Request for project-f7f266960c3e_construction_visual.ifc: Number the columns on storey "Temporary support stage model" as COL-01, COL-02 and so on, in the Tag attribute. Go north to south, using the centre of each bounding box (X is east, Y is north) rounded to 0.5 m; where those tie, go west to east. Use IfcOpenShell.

First a look at what the model holds.

```python
import ifcopenshell
import ifcopenshell.util.element
import ifcopenshell.util.placement

model = ifcopenshell.open("project-f7f266960c3e_construction_visual.ifc")
print(model.schema)
storey = next(s for s in model.by_type("IfcBuildingStorey") if s.Name == "Temporary support stage model")
columns = [e for e in ifcopenshell.util.element.get_decomposition(storey) if e.is_a("IfcColumn")]
for e in sorted(columns, key=lambda e: e.id()):
    origin = ifcopenshell.util.placement.get_local_placement(e.ObjectPlacement)[:3, 3]
    print(e.id(), e.Tag, e.Name, origin.round(2) + 0.0, sep=" | ")
```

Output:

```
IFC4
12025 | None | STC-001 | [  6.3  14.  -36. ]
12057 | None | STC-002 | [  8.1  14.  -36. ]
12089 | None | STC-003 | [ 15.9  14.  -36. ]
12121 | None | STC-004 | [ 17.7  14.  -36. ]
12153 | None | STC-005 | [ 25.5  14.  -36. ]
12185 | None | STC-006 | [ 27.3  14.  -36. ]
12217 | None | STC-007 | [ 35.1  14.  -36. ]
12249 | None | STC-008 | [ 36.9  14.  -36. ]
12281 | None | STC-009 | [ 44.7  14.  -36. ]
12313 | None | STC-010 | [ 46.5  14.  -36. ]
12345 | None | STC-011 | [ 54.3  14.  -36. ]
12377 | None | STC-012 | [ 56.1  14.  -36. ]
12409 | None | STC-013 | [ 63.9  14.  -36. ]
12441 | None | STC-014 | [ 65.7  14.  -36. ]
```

```python
import ifcopenshell
import ifcopenshell.geom
import ifcopenshell.util.element
import ifcopenshell.util.shape

model = ifcopenshell.open("project-f7f266960c3e_construction_visual.ifc")
settings = ifcopenshell.geom.settings()
settings.set("use-world-coords", True)


def centre(element):
    shape = ifcopenshell.geom.create_shape(settings, element)
    return ifcopenshell.util.shape.get_bbox_centroid(shape.geometry)


storey = next(s for s in model.by_type("IfcBuildingStorey") if s.Name == "Temporary support stage model")
columns = [e for e in ifcopenshell.util.element.get_decomposition(storey) if e.is_a("IfcColumn")]

# Insertion points can sit at a corner or the storey origin, so sort by the geometry (in metres).
centres = {e: centre(e) for e in columns}
columns.sort(key=lambda e: (-round(centres[e][1] / 0.5), centres[e][0]))

for i, e in enumerate(columns, start=1):
    number = f"COL-{i:02d}"
    e.Tag = number
    print(e.id(), number)

model.write("project-f7f266960c3e_construction_visual_rev.ifc")
```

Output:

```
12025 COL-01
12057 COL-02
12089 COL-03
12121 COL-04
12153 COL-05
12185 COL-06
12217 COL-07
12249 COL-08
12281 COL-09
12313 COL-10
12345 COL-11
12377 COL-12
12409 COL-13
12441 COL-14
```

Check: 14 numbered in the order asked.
